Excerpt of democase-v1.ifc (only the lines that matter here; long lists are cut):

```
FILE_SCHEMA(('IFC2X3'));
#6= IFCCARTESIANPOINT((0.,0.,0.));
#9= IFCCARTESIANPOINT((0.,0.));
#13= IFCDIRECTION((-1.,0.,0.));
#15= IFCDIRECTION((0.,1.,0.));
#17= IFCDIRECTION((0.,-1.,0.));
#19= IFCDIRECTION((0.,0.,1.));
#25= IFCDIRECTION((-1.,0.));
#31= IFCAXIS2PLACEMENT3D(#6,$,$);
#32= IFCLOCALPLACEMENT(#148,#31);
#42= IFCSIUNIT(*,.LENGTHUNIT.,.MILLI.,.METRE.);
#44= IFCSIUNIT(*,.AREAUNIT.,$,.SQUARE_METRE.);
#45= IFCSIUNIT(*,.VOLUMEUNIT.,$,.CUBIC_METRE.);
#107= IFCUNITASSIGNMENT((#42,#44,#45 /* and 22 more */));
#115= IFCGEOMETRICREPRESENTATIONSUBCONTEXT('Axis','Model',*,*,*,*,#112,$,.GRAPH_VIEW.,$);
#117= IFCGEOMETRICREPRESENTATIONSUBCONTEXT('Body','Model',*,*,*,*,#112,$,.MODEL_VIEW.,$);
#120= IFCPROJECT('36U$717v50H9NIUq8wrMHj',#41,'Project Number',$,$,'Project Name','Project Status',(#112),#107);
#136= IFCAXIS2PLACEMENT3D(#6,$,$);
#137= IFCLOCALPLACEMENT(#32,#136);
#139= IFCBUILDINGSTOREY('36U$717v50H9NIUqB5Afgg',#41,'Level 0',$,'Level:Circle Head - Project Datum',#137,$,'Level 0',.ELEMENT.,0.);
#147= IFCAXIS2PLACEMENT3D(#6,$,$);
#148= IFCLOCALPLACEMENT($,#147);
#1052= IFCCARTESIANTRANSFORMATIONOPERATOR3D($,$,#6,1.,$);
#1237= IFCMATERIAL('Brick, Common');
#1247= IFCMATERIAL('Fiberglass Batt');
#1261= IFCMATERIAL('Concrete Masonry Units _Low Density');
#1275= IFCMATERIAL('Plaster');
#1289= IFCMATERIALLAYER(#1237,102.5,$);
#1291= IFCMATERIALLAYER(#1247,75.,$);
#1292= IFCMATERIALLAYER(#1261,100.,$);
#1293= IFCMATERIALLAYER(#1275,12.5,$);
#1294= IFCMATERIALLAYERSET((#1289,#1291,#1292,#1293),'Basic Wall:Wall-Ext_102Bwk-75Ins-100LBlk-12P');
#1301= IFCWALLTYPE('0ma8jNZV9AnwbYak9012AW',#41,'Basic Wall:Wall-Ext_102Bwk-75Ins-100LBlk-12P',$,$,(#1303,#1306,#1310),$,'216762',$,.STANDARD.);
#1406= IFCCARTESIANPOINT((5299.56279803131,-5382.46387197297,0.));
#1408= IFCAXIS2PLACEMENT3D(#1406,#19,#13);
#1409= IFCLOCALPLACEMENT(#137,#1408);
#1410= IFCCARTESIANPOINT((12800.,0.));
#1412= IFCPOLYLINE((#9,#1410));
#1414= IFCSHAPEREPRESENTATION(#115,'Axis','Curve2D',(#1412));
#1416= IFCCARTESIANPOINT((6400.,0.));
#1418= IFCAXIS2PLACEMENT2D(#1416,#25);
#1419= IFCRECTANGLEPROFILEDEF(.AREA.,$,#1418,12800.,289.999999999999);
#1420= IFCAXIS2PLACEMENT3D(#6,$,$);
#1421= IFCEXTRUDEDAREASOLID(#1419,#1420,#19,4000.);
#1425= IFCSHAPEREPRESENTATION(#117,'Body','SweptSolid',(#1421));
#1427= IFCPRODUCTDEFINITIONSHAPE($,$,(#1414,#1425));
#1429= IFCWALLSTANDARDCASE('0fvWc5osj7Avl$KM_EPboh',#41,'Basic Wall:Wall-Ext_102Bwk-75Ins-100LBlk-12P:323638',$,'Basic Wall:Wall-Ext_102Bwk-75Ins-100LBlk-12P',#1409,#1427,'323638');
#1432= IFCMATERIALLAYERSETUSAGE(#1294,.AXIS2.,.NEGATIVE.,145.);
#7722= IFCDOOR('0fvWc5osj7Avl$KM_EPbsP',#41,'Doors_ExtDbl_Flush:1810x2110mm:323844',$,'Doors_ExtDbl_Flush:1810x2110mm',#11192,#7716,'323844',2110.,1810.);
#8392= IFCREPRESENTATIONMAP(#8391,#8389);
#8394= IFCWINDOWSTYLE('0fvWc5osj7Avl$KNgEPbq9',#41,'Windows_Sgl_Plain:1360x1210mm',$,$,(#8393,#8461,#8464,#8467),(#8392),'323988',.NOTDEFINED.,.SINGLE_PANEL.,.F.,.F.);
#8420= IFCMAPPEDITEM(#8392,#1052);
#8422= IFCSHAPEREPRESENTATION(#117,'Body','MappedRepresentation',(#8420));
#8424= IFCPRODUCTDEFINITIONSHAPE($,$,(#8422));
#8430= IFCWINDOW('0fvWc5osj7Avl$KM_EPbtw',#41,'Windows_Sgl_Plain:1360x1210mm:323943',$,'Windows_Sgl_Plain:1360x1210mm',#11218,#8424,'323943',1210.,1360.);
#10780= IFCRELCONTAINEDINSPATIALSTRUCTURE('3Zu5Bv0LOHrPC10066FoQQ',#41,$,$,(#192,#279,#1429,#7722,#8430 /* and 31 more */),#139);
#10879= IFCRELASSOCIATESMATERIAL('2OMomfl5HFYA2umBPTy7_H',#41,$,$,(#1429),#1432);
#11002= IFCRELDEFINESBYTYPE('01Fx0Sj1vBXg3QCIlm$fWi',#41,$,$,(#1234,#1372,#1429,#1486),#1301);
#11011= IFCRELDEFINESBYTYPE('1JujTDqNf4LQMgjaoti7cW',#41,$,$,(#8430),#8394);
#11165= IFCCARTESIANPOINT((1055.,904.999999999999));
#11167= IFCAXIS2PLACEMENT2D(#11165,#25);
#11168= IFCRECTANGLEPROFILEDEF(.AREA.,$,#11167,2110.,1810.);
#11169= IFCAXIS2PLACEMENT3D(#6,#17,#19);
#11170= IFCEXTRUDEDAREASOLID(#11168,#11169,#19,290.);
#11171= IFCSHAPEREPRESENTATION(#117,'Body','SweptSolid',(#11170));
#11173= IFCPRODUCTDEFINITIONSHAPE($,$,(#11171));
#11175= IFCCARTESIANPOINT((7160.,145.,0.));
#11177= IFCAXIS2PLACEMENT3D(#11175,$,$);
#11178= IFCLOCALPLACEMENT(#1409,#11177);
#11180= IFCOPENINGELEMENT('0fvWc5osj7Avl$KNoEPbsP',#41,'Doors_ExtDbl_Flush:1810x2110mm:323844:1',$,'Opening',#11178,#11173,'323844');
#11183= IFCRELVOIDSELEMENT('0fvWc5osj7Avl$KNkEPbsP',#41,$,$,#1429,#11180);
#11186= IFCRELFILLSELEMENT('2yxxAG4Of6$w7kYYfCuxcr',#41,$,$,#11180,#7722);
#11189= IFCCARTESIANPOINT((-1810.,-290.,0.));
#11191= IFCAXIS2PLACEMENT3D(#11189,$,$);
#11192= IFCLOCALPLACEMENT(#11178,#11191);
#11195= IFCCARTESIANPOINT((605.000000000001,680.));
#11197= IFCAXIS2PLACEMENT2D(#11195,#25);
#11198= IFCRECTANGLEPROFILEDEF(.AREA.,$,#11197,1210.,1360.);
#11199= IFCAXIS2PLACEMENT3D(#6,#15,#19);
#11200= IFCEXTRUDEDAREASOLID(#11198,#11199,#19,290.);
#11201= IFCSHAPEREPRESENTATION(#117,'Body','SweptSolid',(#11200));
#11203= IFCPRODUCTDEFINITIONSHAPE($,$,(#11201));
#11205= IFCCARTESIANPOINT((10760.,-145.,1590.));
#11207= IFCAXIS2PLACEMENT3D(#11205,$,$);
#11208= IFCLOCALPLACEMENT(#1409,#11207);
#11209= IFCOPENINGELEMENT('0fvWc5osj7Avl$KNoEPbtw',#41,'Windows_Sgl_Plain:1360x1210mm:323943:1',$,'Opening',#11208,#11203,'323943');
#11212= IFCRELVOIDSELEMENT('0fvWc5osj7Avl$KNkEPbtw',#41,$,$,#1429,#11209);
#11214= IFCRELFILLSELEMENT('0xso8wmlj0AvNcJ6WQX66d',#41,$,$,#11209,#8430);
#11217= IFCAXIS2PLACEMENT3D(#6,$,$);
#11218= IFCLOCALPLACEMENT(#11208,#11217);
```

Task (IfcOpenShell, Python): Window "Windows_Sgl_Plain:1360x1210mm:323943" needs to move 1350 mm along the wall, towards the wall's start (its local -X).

```python
import ifcopenshell
import ifcopenshell.api.geometry
import ifcopenshell.util.placement

model = ifcopenshell.open("democase-v1.ifc")

window = model.by_guid("0fvWc5osj7Avl$KM_EPbtw")
opening = window.FillsVoids[0].RelatingOpeningElement
wall = opening.VoidsElements[0].RelatingBuildingElement

wall_matrix = ifcopenshell.util.placement.get_local_placement(wall.ObjectPlacement)
shift = wall_matrix[:3, 0] * -1350.0
before = ifcopenshell.util.placement.get_local_placement(window.ObjectPlacement)[:3, 3].copy()

# The window is placed relative to its opening, so it follows when the opening moves.
matrix = ifcopenshell.util.placement.get_local_placement(opening.ObjectPlacement)
matrix[:3, 3] += shift
ifcopenshell.api.geometry.edit_object_placement(
    model, product=opening, matrix=matrix, is_si=False, should_transform_children=True
)

after = ifcopenshell.util.placement.get_local_placement(window.ObjectPlacement)[:3, 3]
print("window moved by", (after - before).round(3) + 0.0)

model.write("democase-v1_updated.ifc")
```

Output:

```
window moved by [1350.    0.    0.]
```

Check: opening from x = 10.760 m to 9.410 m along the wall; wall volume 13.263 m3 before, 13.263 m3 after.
